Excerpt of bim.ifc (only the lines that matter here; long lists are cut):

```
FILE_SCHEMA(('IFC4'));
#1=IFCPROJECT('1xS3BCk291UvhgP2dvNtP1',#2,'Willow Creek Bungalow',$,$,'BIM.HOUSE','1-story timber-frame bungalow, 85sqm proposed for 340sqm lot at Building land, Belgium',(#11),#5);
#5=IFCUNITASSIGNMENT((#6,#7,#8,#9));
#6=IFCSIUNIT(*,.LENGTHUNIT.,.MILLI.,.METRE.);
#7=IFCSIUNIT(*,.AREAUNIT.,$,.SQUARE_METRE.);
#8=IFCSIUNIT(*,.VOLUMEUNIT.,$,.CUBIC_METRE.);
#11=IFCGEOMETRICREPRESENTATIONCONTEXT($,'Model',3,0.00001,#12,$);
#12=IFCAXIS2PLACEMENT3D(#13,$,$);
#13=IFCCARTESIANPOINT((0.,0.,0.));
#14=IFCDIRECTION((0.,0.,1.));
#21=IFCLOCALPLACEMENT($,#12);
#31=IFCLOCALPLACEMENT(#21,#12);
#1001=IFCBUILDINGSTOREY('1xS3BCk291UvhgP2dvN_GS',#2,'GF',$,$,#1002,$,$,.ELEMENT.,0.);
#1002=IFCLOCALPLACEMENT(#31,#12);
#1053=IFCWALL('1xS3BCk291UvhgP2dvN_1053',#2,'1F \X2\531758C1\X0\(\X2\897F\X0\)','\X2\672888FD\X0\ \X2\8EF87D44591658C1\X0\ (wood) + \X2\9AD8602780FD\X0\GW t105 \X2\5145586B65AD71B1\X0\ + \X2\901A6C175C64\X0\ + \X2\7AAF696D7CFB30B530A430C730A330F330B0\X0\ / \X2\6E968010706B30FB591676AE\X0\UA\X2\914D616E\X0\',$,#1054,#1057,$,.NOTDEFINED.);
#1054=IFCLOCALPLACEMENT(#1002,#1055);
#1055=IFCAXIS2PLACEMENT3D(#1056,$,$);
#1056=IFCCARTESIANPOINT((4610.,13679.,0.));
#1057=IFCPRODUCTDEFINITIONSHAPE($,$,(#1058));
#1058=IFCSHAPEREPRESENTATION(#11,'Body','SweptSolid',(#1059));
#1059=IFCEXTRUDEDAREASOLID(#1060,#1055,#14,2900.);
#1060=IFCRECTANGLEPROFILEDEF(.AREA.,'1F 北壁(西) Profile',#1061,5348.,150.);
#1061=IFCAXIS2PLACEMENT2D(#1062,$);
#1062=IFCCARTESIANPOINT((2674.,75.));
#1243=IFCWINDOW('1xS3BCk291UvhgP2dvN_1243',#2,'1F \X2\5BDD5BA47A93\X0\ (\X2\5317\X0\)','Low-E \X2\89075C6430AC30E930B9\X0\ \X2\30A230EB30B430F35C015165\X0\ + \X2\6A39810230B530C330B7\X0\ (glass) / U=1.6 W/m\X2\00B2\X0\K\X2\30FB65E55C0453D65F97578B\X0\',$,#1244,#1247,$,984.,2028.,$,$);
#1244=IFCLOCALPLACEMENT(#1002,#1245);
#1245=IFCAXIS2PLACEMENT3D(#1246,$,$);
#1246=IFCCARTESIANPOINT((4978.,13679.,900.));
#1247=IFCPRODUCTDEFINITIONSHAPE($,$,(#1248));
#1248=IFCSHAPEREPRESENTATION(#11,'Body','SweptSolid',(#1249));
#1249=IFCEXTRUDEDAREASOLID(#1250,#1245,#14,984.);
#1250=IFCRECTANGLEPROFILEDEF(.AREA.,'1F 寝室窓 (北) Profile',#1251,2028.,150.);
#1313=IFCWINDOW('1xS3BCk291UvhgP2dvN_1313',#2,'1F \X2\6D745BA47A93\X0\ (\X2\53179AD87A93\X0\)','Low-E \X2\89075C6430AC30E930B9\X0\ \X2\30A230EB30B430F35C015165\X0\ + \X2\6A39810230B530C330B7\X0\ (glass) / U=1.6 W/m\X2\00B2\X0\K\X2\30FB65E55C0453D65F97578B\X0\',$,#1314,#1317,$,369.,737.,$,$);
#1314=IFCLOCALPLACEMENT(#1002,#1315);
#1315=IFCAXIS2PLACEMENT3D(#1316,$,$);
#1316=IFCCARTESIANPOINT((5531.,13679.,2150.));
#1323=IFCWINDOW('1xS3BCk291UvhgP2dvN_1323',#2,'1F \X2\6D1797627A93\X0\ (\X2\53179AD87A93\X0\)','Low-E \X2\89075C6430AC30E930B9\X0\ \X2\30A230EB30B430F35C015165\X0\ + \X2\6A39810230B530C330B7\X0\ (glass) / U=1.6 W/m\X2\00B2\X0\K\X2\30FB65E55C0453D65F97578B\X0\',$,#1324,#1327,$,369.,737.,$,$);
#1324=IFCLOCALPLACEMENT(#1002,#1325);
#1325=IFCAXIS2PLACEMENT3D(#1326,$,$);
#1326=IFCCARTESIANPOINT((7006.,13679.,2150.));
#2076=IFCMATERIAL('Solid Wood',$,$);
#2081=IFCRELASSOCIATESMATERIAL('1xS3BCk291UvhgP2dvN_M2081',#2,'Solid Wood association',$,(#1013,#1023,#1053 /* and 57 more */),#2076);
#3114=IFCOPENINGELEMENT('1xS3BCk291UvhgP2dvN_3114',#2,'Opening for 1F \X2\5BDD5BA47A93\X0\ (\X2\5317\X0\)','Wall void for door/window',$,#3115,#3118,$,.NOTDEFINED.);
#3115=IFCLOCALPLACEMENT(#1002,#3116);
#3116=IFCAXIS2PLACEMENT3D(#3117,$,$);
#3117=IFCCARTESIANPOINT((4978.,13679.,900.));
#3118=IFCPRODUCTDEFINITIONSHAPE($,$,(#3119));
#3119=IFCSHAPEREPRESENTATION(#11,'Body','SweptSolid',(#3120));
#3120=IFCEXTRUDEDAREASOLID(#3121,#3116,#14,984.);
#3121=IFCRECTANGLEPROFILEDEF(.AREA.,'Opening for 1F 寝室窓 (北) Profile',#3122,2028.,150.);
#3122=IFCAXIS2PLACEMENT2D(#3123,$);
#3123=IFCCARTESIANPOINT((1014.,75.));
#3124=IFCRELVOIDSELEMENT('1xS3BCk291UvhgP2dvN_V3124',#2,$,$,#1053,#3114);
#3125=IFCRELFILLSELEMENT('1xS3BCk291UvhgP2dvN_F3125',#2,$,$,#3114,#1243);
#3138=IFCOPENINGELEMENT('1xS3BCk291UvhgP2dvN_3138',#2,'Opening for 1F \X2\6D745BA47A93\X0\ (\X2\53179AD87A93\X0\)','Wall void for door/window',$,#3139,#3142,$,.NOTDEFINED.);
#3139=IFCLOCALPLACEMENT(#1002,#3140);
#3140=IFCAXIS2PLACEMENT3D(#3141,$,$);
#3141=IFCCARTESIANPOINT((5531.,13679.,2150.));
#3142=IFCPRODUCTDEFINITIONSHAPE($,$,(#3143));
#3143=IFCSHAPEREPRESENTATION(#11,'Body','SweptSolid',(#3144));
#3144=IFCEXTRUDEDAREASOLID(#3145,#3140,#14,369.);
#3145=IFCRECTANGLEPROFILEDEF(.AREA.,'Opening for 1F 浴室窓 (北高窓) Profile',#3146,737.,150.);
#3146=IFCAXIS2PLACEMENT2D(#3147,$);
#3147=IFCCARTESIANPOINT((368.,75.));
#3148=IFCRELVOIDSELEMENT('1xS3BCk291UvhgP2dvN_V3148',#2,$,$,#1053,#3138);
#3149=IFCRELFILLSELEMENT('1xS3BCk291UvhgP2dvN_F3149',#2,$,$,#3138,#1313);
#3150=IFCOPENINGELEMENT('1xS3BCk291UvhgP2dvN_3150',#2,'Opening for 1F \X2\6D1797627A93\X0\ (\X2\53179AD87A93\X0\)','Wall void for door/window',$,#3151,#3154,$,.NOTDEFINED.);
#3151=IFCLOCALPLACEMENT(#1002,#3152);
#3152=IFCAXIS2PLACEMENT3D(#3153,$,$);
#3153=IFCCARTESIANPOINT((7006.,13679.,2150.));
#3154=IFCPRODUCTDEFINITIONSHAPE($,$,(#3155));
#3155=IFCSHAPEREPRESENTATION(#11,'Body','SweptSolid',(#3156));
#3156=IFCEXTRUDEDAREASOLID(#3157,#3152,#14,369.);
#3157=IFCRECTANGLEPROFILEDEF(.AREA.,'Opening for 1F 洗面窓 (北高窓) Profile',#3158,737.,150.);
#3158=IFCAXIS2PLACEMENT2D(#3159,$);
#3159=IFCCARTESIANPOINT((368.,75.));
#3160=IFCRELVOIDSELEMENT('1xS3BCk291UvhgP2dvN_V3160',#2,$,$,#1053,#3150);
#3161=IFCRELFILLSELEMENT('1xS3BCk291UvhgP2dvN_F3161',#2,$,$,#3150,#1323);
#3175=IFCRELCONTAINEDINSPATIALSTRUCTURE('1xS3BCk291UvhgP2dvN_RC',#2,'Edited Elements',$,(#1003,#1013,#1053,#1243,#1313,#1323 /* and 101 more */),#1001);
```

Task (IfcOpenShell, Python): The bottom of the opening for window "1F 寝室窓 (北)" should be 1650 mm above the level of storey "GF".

```python
import numpy as np
import ifcopenshell
import ifcopenshell.api.geometry
import ifcopenshell.geom
import ifcopenshell.util.element
import ifcopenshell.util.placement
import ifcopenshell.util.shape
import ifcopenshell.util.unit

model = ifcopenshell.open("bim.ifc")
unit_scale = ifcopenshell.util.unit.calculate_unit_scale(model)

window = model.by_guid("1xS3BCk291UvhgP2dvN_1243")
opening = window.FillsVoids[0].RelatingOpeningElement
storey = ifcopenshell.util.element.get_container(window, ifc_class="IfcBuildingStorey")
level = ifcopenshell.util.placement.get_local_placement(storey.ObjectPlacement)[2, 3]

# The opening's origin need not be at the sill, so measure its lowest point.
shape = ifcopenshell.geom.create_shape(ifcopenshell.geom.settings(), opening)
bottom = ifcopenshell.util.shape.get_shape_bottom_elevation(shape, shape.geometry) / unit_scale
dz = level + 1650.0 - bottom

shift = np.array([0.0, 0.0, dz])
# The window is not placed relative to its opening, so move both.
for product in (opening, window):
    matrix = ifcopenshell.util.placement.get_local_placement(product.ObjectPlacement)
    matrix[:3, 3] += shift
    ifcopenshell.api.geometry.edit_object_placement(model, product=product, matrix=matrix, is_si=False)

print(f"moved by {dz * unit_scale:+.3f} m")

model.write("bim_edited.ifc")
```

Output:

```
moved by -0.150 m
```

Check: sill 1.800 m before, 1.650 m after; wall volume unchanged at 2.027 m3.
